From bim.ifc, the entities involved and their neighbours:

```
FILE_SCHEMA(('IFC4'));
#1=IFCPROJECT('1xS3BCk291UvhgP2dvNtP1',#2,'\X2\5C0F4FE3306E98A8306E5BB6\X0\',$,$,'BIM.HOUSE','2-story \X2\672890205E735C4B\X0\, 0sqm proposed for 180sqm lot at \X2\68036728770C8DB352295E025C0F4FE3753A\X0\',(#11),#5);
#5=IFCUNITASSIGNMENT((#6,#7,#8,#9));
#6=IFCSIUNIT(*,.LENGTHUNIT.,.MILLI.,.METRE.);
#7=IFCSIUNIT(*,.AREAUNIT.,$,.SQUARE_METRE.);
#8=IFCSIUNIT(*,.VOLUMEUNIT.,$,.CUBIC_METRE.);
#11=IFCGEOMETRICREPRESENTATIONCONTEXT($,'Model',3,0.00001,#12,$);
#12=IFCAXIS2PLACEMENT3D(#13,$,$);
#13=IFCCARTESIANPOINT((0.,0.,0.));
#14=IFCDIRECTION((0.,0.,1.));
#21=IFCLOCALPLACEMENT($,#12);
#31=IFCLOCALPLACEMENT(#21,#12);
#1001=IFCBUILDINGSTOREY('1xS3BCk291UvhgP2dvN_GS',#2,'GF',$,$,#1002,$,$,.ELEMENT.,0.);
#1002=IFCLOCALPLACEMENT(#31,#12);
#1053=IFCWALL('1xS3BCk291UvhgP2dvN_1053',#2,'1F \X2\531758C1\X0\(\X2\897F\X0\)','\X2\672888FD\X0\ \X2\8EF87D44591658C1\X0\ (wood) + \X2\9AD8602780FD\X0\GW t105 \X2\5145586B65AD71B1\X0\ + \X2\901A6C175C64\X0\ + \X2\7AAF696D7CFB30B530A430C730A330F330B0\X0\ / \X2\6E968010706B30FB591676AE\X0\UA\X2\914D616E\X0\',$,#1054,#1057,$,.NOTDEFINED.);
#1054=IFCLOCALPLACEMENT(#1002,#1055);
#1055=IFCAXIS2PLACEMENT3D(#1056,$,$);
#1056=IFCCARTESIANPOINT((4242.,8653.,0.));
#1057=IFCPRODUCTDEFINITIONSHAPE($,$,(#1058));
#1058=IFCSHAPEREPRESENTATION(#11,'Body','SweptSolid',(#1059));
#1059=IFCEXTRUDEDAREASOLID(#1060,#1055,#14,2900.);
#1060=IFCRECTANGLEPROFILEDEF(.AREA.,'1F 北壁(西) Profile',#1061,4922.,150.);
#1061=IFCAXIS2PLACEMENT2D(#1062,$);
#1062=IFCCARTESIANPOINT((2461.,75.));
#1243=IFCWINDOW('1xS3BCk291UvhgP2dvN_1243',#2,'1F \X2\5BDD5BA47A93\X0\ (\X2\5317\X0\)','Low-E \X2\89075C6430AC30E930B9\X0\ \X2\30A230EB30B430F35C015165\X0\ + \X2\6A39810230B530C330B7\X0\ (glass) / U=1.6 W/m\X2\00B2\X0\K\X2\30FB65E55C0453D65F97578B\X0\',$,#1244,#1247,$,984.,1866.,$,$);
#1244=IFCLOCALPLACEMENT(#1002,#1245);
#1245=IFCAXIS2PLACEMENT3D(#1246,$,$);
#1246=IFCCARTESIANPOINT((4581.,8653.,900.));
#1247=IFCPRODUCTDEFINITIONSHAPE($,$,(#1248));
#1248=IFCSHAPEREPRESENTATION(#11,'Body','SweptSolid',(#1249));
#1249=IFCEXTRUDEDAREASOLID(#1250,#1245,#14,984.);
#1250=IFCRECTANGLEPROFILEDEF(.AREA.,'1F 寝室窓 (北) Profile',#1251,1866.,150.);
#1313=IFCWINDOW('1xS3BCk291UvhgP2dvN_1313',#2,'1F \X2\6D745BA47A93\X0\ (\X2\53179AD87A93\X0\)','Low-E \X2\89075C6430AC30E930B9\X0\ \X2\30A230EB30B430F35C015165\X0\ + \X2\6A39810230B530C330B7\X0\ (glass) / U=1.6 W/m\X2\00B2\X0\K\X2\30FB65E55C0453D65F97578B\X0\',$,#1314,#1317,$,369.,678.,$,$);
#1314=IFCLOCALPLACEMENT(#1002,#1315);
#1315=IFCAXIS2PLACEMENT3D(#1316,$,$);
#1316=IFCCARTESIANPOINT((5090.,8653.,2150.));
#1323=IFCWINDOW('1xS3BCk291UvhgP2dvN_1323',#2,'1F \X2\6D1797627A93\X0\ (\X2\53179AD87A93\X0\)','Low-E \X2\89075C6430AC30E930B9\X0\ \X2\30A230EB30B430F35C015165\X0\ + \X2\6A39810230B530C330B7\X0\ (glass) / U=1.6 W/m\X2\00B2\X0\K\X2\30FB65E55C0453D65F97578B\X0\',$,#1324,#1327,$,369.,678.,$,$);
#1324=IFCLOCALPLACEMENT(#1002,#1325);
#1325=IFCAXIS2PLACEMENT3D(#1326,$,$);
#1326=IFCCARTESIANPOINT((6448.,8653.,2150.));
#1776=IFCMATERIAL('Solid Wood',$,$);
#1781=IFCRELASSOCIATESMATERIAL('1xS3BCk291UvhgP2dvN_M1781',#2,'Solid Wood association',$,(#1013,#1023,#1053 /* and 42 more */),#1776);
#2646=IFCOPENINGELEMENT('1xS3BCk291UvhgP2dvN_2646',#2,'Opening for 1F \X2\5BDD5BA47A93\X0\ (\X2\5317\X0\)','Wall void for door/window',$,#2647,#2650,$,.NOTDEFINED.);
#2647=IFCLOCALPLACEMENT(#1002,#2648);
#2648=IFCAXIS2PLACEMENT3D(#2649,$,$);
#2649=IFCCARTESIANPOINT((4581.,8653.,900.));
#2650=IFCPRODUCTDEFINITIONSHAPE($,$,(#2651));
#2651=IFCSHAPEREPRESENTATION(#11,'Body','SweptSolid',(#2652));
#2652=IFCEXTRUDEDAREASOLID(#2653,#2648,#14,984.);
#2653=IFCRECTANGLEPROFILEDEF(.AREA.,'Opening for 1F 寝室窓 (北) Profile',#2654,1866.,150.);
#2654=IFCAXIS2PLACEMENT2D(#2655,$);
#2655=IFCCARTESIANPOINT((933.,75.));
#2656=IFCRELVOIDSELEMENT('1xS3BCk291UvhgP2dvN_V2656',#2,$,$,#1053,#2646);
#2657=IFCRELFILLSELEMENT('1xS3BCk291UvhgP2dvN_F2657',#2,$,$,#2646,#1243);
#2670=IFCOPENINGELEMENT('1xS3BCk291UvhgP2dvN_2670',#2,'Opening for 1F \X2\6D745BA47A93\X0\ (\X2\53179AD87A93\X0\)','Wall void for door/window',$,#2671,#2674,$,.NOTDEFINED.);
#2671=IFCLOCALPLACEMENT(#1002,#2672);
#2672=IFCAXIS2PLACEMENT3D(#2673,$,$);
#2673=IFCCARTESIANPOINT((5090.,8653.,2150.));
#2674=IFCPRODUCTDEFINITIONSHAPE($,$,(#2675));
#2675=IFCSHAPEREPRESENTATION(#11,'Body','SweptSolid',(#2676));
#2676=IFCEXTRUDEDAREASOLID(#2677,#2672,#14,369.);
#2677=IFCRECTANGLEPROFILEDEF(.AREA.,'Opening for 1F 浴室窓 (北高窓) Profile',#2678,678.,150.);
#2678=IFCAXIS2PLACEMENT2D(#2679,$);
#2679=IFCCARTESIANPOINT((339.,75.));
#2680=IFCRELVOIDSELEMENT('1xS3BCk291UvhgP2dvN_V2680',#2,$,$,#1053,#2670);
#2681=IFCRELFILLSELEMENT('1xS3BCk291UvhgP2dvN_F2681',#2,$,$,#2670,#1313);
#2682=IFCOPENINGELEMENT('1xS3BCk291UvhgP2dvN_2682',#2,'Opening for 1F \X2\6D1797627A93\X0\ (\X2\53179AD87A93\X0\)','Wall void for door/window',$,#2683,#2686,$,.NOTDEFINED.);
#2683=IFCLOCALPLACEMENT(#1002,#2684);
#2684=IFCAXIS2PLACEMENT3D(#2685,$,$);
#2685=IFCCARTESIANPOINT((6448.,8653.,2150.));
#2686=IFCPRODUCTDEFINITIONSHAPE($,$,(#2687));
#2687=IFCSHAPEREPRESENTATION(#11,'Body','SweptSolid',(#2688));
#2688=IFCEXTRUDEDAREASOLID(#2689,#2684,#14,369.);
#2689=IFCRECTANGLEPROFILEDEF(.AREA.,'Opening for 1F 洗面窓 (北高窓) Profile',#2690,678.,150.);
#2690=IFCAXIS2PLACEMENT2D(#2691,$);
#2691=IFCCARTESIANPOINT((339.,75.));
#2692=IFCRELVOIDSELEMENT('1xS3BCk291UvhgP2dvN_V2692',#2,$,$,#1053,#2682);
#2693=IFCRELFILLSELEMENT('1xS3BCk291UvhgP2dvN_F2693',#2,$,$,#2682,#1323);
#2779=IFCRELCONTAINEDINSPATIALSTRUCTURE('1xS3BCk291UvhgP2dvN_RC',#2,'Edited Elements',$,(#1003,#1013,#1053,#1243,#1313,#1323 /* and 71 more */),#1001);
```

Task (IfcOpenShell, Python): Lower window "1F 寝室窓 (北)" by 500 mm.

```python
import numpy as np
import ifcopenshell
import ifcopenshell.api.geometry
import ifcopenshell.util.placement
import ifcopenshell.util.unit

model = ifcopenshell.open("bim.ifc")
unit_scale = ifcopenshell.util.unit.calculate_unit_scale(model)

window = model.by_guid("1xS3BCk291UvhgP2dvN_1243")
opening = window.FillsVoids[0].RelatingOpeningElement
dz = -0.5 / unit_scale

shift = np.array([0.0, 0.0, dz])
# The window is not placed relative to its opening, so move both.
for product in (opening, window):
    matrix = ifcopenshell.util.placement.get_local_placement(product.ObjectPlacement)
    matrix[:3, 3] += shift
    ifcopenshell.api.geometry.edit_object_placement(model, product=product, matrix=matrix, is_si=False)

print(f"moved by {dz * unit_scale:+.3f} m")

model.write("bim_rev.ifc")
```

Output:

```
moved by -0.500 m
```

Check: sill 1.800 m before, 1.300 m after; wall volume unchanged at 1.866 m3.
